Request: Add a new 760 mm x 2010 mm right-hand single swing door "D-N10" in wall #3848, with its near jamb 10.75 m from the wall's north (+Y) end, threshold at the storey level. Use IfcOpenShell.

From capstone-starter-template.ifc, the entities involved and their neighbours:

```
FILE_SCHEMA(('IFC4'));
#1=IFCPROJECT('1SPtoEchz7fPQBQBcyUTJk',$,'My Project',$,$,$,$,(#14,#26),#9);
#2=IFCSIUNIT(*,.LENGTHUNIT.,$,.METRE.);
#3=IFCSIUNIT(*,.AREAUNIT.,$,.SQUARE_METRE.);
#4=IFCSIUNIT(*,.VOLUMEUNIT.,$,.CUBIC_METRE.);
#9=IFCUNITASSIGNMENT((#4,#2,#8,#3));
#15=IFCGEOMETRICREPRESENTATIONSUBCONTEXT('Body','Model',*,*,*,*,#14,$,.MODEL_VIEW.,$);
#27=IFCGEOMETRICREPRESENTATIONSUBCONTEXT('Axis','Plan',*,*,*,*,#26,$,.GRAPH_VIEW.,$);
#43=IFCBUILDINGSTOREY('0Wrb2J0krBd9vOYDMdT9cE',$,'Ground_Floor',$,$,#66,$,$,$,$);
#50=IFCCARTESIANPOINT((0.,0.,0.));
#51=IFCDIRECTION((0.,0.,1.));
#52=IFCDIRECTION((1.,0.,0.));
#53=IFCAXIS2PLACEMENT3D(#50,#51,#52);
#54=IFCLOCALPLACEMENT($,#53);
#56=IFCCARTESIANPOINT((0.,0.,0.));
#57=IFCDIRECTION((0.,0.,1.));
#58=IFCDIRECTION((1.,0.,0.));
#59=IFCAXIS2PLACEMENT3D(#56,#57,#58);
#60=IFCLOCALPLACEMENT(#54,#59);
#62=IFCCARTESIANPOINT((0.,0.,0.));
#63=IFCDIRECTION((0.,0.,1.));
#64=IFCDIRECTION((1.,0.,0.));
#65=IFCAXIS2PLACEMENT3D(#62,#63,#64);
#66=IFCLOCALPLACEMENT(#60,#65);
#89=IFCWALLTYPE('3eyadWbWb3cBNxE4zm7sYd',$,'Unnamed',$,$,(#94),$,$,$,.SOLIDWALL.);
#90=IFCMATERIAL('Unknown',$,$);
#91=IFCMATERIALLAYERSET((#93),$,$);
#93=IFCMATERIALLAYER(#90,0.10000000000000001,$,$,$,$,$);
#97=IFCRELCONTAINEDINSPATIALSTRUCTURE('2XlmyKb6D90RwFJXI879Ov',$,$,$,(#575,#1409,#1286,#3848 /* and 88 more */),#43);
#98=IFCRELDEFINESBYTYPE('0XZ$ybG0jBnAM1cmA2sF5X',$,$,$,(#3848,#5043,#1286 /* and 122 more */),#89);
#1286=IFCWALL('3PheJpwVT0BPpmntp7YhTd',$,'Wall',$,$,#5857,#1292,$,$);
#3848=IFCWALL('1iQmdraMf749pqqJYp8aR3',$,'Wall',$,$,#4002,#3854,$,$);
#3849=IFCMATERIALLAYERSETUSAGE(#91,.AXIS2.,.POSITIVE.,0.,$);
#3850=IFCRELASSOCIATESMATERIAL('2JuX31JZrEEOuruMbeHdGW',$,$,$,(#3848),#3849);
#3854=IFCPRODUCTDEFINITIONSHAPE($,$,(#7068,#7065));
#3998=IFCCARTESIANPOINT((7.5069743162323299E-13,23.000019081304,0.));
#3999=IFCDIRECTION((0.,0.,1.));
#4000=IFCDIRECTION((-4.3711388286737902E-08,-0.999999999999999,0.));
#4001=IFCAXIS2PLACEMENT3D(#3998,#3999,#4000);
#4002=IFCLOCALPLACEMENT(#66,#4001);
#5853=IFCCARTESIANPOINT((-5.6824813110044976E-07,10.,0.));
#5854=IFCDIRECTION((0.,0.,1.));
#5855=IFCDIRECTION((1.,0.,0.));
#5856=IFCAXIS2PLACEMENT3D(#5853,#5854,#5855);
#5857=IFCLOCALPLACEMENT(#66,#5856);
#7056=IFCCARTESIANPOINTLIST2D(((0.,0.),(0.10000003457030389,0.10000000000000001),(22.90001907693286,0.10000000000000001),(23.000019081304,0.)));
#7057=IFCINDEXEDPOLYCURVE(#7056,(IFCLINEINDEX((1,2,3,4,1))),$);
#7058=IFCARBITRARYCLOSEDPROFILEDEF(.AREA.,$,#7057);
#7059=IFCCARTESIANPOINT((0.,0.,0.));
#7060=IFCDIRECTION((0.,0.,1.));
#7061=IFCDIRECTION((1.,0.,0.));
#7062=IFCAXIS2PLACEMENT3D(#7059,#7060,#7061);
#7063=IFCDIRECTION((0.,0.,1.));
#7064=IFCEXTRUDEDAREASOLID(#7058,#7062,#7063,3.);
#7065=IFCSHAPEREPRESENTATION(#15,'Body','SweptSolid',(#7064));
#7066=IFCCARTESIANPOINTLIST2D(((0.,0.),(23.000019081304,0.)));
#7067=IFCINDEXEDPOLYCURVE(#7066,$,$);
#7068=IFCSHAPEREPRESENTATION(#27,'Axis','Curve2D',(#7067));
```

```python
import numpy as np
import ifcopenshell
import ifcopenshell.api.feature
import ifcopenshell.api.geometry
import ifcopenshell.api.root
import ifcopenshell.api.spatial
import ifcopenshell.geom
import ifcopenshell.util.element
import ifcopenshell.util.placement
import ifcopenshell.util.representation
import ifcopenshell.util.shape
import ifcopenshell.util.unit

model = ifcopenshell.open("capstone-starter-template.ifc")
unit_scale = ifcopenshell.util.unit.calculate_unit_scale(model)
settings = ifcopenshell.geom.settings()


def volume(element):
    """Net volume in cubic metres, openings subtracted."""
    shape = ifcopenshell.geom.create_shape(settings, element)
    return ifcopenshell.util.shape.get_volume(shape.geometry)


wall = model.by_id(3848)
storey = ifcopenshell.util.element.get_container(wall, ifc_class="IfcBuildingStorey")
context = ifcopenshell.util.representation.get_context(model, "Model", "Body", "MODEL_VIEW")
before = volume(wall)

width, height, from_end, sill = 0.76, 2.01, 10.75, 0.0  # metres

# The wall runs along its own X axis, and the end named is its -X end.
wall_shape = ifcopenshell.geom.create_shape(settings, wall)
x, y, z = ifcopenshell.util.shape.get_vertices(wall_shape.geometry).T
start = x.min() + from_end
face, thickness = float(y.min()), float(y.max() - y.min())
wall_matrix = ifcopenshell.util.placement.get_local_placement(wall.ObjectPlacement)
level = ifcopenshell.util.placement.get_local_placement(storey.ObjectPlacement)[2, 3]


def in_wall(x, y):
    """Placement at x, y metres in the wall's axes, at sill height."""
    matrix = wall_matrix.copy()
    matrix[:, 3] = wall_matrix @ np.array([x / unit_scale, y / unit_scale, 0.0, 1.0])
    matrix[2, 3] = level + sill / unit_scale
    return matrix


# Opening: a box that overshoots both wall faces by 50 mm.
opening = ifcopenshell.api.root.create_entity(model, ifc_class="IfcOpeningElement", predefined_type="OPENING")
box = ifcopenshell.api.geometry.add_wall_representation(
    model, context=context, length=width, height=height, thickness=thickness + 0.1
)
ifcopenshell.api.geometry.assign_representation(model, product=opening, representation=box)
ifcopenshell.api.geometry.edit_object_placement(model, product=opening, matrix=in_wall(start, face - 0.05), is_si=False)
ifcopenshell.api.feature.add_feature(model, feature=opening, element=wall)

door = ifcopenshell.api.root.create_entity(model, ifc_class="IfcDoor", name="D-N10", predefined_type="DOOR")
door.OverallWidth, door.OverallHeight = width / unit_scale, height / unit_scale
door.OperationType = "SINGLE_SWING_RIGHT"
body = ifcopenshell.api.geometry.add_door_representation(
    model,
    context=context,
    overall_width=door.OverallWidth,
    overall_height=door.OverallHeight,
    operation_type="SINGLE_SWING_RIGHT",
    lining_properties={"LiningDepth": thickness / unit_scale, "ThresholdDepth": thickness / unit_scale},
)
ifcopenshell.api.geometry.assign_representation(model, product=door, representation=body)
ifcopenshell.api.spatial.assign_container(model, products=[door], relating_structure=storey)
ifcopenshell.api.feature.add_filling(model, opening=opening, element=door)

# The lining spans the wall, so the door starts at the wall face.
ifcopenshell.api.geometry.edit_object_placement(model, product=door, matrix=in_wall(start, face), is_si=False)

after = volume(wall)

print(f"wall volume {before:.3f} -> {after:.3f} m3")

model.write("capstone-starter-template_edited.ifc")
```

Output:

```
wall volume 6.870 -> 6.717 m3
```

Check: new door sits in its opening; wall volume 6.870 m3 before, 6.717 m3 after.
